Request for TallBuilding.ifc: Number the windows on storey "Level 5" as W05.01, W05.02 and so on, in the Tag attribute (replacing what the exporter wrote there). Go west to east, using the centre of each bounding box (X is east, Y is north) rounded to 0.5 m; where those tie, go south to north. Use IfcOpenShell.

First a look at what the model holds.

```python
import ifcopenshell
import ifcopenshell.util.element
import ifcopenshell.util.placement

model = ifcopenshell.open("TallBuilding.ifc")
print(model.schema)
storey = next(s for s in model.by_type("IfcBuildingStorey") if s.Name == "Level 5")
windows = [e for e in ifcopenshell.util.element.get_decomposition(storey) if e.is_a("IfcWindow")]
for e in sorted(windows, key=lambda e: e.id()):
    origin = ifcopenshell.util.placement.get_local_placement(e.ObjectPlacement)[:3, 3]
    print(e.id(), e.Tag, e.Name, origin.round(2) + 0.0, sep=" | ")
```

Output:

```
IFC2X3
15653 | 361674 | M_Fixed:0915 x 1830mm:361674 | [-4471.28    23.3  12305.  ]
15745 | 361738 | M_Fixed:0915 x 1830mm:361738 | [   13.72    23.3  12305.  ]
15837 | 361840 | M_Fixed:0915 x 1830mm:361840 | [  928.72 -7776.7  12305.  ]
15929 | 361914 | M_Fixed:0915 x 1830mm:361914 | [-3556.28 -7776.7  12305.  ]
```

```python
import ifcopenshell
import ifcopenshell.geom
import ifcopenshell.util.element
import ifcopenshell.util.shape

model = ifcopenshell.open("TallBuilding.ifc")
settings = ifcopenshell.geom.settings()
settings.set("use-world-coords", True)


def centre(element):
    shape = ifcopenshell.geom.create_shape(settings, element)
    return ifcopenshell.util.shape.get_bbox_centroid(shape.geometry)


storey = next(s for s in model.by_type("IfcBuildingStorey") if s.Name == "Level 5")
windows = [e for e in ifcopenshell.util.element.get_decomposition(storey) if e.is_a("IfcWindow")]

# Insertion points can sit at a corner or the storey origin, so sort by the geometry (in metres).
centres = {e: centre(e) for e in windows}
windows.sort(key=lambda e: (round(centres[e][0] / 0.5), centres[e][1]))

for i, e in enumerate(windows, start=1):
    number = f"W05.{i:02d}"
    e.Tag = number
    print(e.id(), number)

model.write("TallBuilding_edited.ifc")
```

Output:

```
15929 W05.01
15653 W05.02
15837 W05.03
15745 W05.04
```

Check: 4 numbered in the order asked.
